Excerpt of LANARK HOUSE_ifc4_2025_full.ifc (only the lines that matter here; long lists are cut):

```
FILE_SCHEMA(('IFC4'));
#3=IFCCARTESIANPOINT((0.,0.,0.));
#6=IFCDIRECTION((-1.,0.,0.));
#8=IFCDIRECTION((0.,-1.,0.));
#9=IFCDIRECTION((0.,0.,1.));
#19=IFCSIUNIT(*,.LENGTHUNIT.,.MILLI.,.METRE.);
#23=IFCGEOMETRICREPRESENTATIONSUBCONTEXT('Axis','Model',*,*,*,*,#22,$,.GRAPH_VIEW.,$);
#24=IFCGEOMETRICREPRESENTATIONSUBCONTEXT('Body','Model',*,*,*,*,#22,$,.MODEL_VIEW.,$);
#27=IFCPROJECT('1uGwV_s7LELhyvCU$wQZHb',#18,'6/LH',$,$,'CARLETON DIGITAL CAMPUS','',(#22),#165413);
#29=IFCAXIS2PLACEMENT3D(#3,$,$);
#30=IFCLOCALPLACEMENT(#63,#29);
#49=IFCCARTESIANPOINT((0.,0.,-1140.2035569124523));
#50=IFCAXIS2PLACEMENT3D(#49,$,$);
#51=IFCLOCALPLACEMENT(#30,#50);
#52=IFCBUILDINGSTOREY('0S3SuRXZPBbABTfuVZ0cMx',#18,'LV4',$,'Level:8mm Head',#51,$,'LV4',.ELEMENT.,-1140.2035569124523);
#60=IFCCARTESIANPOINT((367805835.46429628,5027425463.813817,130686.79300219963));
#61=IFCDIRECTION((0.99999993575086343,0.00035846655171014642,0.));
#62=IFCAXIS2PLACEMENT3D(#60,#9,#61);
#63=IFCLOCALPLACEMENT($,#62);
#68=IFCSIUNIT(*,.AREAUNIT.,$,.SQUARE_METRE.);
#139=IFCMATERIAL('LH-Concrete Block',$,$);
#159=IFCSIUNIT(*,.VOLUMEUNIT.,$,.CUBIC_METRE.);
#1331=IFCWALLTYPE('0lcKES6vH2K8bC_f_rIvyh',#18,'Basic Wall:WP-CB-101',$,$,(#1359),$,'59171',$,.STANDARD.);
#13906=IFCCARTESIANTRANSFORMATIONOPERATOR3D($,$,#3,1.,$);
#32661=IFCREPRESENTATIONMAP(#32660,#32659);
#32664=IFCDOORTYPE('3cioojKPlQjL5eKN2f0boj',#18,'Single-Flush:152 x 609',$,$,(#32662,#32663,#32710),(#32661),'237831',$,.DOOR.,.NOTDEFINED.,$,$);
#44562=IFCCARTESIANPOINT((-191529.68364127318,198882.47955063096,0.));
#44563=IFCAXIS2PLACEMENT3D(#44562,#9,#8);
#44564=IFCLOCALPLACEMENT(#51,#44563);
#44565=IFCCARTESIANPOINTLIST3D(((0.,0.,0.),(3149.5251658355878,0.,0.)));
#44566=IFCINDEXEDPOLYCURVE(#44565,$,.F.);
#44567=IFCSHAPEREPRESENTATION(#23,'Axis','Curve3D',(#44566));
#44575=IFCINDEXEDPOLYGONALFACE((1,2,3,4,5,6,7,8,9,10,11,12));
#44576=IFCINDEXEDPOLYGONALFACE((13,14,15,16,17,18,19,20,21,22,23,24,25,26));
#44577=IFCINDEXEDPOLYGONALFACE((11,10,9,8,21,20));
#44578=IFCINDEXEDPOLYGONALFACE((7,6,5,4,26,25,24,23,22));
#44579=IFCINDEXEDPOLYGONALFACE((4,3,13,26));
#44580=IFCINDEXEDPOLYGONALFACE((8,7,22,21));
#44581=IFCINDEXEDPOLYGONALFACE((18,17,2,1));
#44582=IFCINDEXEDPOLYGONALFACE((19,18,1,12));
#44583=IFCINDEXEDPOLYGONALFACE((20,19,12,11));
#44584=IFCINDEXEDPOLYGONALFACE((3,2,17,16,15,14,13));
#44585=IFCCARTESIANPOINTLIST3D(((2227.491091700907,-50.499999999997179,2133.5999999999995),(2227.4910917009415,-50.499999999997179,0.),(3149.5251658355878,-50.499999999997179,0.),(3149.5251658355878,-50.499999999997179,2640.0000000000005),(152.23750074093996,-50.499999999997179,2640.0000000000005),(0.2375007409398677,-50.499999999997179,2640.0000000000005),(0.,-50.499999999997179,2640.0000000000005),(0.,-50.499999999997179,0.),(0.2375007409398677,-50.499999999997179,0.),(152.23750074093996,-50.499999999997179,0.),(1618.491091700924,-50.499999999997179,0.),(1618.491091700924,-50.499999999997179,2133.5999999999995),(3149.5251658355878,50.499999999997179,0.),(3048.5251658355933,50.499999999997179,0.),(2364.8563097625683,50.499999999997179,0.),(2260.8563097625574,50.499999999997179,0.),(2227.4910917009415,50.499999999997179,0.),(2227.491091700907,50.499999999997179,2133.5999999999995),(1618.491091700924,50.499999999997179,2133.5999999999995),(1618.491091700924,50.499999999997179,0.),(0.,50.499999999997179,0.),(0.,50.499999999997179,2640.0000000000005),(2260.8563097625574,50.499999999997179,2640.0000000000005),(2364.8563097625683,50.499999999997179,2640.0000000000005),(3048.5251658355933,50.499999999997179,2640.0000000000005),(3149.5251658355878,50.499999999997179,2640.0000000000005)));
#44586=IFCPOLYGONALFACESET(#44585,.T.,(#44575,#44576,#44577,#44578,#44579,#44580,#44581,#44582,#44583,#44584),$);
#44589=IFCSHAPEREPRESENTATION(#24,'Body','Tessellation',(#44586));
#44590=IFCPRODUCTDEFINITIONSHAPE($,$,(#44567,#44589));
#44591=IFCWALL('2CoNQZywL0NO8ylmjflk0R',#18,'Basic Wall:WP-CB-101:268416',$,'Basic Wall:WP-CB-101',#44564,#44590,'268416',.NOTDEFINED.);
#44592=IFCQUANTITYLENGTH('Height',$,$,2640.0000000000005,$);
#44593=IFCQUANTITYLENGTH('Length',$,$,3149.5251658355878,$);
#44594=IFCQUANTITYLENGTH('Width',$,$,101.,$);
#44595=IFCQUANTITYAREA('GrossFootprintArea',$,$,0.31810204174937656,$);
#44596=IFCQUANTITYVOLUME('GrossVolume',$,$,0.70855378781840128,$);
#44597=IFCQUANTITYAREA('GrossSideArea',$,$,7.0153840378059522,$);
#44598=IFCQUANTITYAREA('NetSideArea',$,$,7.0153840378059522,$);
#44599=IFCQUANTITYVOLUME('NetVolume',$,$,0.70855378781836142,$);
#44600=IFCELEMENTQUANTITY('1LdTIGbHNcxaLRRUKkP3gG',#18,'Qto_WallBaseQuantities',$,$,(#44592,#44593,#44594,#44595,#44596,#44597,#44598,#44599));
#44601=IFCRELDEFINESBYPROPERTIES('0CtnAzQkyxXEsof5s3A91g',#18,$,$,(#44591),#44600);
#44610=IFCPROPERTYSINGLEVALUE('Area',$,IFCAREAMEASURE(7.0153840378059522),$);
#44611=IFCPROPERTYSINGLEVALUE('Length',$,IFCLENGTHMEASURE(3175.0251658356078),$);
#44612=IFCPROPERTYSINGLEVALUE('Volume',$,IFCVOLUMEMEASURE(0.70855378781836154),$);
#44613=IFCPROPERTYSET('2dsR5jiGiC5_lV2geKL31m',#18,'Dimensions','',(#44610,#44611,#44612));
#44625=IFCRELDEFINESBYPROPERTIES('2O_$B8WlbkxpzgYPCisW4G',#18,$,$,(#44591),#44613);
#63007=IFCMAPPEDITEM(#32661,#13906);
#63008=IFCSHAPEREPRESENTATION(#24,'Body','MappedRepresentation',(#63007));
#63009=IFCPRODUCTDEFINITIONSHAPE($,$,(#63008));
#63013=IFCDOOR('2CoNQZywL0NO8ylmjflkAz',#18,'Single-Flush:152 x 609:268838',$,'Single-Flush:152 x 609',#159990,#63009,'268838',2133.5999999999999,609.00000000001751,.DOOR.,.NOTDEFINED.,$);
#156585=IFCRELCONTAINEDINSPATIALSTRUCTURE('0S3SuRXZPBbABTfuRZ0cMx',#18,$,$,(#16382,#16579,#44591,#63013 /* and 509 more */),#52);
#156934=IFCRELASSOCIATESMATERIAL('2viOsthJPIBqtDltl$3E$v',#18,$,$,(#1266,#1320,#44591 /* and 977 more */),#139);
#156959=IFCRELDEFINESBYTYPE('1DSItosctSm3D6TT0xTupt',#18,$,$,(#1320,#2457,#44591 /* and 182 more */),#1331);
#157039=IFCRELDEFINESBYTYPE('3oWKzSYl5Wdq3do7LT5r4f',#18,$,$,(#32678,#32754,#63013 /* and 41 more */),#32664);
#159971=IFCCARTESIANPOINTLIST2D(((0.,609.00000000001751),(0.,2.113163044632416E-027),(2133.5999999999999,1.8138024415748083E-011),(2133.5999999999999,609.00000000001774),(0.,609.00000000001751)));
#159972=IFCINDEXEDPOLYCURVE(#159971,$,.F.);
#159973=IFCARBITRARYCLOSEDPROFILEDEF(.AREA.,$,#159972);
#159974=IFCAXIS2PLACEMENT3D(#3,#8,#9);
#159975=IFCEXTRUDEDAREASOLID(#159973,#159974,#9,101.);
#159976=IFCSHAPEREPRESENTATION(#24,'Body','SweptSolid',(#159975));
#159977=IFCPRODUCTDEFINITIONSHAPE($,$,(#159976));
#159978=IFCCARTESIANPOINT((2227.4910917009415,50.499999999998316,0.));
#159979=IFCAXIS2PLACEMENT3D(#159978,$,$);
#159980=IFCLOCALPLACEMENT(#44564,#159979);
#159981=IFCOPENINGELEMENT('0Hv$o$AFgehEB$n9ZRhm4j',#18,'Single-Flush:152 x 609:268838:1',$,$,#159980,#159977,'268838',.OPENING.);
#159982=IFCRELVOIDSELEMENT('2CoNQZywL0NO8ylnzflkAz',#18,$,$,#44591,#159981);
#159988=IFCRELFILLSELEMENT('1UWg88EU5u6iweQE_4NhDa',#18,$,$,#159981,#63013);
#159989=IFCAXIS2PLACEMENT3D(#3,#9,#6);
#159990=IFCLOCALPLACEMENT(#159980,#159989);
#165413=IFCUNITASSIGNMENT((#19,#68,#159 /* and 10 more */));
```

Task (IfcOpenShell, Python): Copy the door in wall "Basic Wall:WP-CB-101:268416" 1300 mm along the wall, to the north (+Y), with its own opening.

```python
import ifcopenshell
import ifcopenshell.api.feature
import ifcopenshell.api.geometry
import ifcopenshell.api.pset
import ifcopenshell.api.root
import ifcopenshell.geom
import ifcopenshell.util.element
import ifcopenshell.util.placement
import ifcopenshell.util.shape
import ifcopenshell.util.unit

model = ifcopenshell.open("LANARK HOUSE_ifc4_2025_full.ifc")
unit_scale = ifcopenshell.util.unit.calculate_unit_scale(model)
area_scale = ifcopenshell.util.unit.calculate_unit_scale(model, "AREAUNIT")
volume_scale = ifcopenshell.util.unit.calculate_unit_scale(model, "VOLUMEUNIT")
settings = ifcopenshell.geom.settings()


def volume(element):
    """Net volume in cubic metres, openings subtracted."""
    shape = ifcopenshell.geom.create_shape(settings, element)
    return ifcopenshell.util.shape.get_volume(shape.geometry)


def reuse_history(source, copy):
    """copy_class also copies each property set's owner history, people and application; keep the originals."""
    for rel in copy.IsDefinedBy:
        if rel.is_a("IfcRelDefinesByProperties") and (history := rel.RelatingPropertyDefinition.OwnerHistory):
            rel.RelatingPropertyDefinition.OwnerHistory = source.OwnerHistory
            ifcopenshell.util.element.remove_deep2(model, history)


door = model.by_id(63013)
opening = door.FillsVoids[0].RelatingOpeningElement
wall = opening.VoidsElements[0].RelatingBuildingElement
before = volume(wall)
shift = ifcopenshell.util.placement.get_local_placement(wall.ObjectPlacement)[:3, 0] * -1.3 / unit_scale

# copy_class copies the void relationship, type, container and properties, but no geometry.
new_opening = ifcopenshell.api.root.copy_class(model, product=opening)
new_opening.Representation = ifcopenshell.util.element.copy_deep(
    model, opening.Representation, exclude=["IfcGeometricRepresentationContext", "IfcRepresentationMap"]
)
new_opening.Name = "Single-Flush:152 x 609"
new_opening.Tag = None
reuse_history(opening, new_opening)
new_door = ifcopenshell.api.root.copy_class(model, product=door)
new_door.Representation = ifcopenshell.util.element.copy_deep(
    model, door.Representation, exclude=["IfcGeometricRepresentationContext", "IfcRepresentationMap"]
)
new_door.Name = "Single-Flush:152 x 609"
new_door.Tag = None
reuse_history(door, new_door)
ifcopenshell.api.feature.add_filling(model, opening=new_opening, element=new_door)

for old, new in ((opening, new_opening), (door, new_door)):
    matrix = ifcopenshell.util.placement.get_local_placement(old.ObjectPlacement)
    matrix[:3, 3] += shift
    ifcopenshell.api.geometry.edit_object_placement(model, product=new, matrix=matrix, is_si=False)

after = volume(wall)
thickness = 0.101  # wall thickness in metres

# Update the wall's stored quantities.
qto = model.by_id(ifcopenshell.util.element.get_pset(wall, "Qto_WallBaseQuantities", should_inherit=False)["id"])
ifcopenshell.api.pset.edit_qto(model, qto=qto, properties={
    "NetSideArea": after / thickness / area_scale,
    "NetVolume": after / volume_scale,
})
pset = model.by_id(ifcopenshell.util.element.get_pset(wall, "Dimensions", should_inherit=False)["id"])
ifcopenshell.api.pset.edit_pset(model, pset=pset, properties={
    "Area": model.create_entity("IfcAreaMeasure", after / thickness / area_scale),
    "Volume": model.create_entity("IfcVolumeMeasure", after / volume_scale),
})

print(f"wall volume {before:.3f} -> {after:.3f} m3")

model.write("LANARK HOUSE_ifc4_2025_full_v2.ifc")
```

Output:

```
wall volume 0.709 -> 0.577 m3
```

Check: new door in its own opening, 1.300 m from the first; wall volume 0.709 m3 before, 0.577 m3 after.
